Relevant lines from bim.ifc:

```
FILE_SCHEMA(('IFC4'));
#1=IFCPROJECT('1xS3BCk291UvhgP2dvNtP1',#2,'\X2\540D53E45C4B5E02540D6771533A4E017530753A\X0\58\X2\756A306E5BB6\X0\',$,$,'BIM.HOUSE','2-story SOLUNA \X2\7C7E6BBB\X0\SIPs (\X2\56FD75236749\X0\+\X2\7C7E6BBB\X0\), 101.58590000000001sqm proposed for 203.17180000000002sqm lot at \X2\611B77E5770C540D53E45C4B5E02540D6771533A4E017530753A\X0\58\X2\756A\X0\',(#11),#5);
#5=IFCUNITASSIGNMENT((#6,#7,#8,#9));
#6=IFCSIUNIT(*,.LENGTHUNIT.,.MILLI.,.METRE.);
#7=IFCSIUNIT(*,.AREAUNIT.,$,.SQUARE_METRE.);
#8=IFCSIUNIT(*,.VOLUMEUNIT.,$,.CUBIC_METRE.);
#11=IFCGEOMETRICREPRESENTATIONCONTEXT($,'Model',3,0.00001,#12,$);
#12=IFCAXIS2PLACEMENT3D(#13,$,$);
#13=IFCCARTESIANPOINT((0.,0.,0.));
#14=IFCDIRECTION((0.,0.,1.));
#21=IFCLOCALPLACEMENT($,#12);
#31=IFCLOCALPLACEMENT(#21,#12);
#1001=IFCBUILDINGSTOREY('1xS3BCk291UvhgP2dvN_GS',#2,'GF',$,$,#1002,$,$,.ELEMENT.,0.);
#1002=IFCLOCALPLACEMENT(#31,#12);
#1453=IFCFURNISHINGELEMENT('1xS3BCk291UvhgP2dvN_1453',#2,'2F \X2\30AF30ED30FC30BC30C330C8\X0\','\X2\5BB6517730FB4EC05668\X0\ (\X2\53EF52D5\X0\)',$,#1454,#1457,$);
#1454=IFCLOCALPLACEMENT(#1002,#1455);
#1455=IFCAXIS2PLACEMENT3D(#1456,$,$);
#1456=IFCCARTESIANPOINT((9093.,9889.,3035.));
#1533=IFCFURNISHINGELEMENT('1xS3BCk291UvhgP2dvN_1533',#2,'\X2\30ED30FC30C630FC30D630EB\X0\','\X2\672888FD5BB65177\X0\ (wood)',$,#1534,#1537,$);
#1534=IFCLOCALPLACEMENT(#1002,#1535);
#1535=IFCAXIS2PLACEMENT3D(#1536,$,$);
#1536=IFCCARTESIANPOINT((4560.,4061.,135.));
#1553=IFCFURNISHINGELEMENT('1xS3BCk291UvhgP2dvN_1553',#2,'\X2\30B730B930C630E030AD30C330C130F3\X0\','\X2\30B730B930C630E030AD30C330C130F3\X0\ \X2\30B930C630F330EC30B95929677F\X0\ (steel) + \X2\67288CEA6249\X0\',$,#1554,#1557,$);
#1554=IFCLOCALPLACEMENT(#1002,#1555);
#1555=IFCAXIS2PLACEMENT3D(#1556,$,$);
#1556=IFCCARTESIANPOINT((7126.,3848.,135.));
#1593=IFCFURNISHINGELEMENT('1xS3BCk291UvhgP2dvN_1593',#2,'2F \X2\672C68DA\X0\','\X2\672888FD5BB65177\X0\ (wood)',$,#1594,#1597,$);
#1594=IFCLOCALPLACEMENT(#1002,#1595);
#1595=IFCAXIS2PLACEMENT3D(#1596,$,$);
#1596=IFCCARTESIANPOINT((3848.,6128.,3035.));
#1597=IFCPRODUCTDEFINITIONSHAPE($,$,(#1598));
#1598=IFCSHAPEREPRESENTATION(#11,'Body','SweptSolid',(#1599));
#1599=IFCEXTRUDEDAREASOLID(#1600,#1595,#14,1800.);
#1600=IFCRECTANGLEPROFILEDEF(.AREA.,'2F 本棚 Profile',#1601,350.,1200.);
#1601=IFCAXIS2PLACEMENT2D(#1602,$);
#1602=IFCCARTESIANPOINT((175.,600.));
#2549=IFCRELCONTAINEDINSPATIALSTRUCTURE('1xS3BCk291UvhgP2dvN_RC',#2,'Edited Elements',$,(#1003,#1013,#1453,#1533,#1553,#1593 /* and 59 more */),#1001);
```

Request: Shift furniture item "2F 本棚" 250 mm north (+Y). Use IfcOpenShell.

```python
import ifcopenshell
import ifcopenshell.api.geometry
import ifcopenshell.util.placement
import ifcopenshell.util.unit

model = ifcopenshell.open("bim.ifc")
unit_scale = ifcopenshell.util.unit.calculate_unit_scale(model)

item = model.by_id(1593)
matrix = ifcopenshell.util.placement.get_local_placement(item.ObjectPlacement)
matrix[1, 3] += 0.25 / unit_scale
ifcopenshell.api.geometry.edit_object_placement(model, product=item, matrix=matrix, is_si=False)

print(ifcopenshell.util.placement.get_local_placement(item.ObjectPlacement).round(3) + 0.0)

model.write("bim_v2.ifc")
```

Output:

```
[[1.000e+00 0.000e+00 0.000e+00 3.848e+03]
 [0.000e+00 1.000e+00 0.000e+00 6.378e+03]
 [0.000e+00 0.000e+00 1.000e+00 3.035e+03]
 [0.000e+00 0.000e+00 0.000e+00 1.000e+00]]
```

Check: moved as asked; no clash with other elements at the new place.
